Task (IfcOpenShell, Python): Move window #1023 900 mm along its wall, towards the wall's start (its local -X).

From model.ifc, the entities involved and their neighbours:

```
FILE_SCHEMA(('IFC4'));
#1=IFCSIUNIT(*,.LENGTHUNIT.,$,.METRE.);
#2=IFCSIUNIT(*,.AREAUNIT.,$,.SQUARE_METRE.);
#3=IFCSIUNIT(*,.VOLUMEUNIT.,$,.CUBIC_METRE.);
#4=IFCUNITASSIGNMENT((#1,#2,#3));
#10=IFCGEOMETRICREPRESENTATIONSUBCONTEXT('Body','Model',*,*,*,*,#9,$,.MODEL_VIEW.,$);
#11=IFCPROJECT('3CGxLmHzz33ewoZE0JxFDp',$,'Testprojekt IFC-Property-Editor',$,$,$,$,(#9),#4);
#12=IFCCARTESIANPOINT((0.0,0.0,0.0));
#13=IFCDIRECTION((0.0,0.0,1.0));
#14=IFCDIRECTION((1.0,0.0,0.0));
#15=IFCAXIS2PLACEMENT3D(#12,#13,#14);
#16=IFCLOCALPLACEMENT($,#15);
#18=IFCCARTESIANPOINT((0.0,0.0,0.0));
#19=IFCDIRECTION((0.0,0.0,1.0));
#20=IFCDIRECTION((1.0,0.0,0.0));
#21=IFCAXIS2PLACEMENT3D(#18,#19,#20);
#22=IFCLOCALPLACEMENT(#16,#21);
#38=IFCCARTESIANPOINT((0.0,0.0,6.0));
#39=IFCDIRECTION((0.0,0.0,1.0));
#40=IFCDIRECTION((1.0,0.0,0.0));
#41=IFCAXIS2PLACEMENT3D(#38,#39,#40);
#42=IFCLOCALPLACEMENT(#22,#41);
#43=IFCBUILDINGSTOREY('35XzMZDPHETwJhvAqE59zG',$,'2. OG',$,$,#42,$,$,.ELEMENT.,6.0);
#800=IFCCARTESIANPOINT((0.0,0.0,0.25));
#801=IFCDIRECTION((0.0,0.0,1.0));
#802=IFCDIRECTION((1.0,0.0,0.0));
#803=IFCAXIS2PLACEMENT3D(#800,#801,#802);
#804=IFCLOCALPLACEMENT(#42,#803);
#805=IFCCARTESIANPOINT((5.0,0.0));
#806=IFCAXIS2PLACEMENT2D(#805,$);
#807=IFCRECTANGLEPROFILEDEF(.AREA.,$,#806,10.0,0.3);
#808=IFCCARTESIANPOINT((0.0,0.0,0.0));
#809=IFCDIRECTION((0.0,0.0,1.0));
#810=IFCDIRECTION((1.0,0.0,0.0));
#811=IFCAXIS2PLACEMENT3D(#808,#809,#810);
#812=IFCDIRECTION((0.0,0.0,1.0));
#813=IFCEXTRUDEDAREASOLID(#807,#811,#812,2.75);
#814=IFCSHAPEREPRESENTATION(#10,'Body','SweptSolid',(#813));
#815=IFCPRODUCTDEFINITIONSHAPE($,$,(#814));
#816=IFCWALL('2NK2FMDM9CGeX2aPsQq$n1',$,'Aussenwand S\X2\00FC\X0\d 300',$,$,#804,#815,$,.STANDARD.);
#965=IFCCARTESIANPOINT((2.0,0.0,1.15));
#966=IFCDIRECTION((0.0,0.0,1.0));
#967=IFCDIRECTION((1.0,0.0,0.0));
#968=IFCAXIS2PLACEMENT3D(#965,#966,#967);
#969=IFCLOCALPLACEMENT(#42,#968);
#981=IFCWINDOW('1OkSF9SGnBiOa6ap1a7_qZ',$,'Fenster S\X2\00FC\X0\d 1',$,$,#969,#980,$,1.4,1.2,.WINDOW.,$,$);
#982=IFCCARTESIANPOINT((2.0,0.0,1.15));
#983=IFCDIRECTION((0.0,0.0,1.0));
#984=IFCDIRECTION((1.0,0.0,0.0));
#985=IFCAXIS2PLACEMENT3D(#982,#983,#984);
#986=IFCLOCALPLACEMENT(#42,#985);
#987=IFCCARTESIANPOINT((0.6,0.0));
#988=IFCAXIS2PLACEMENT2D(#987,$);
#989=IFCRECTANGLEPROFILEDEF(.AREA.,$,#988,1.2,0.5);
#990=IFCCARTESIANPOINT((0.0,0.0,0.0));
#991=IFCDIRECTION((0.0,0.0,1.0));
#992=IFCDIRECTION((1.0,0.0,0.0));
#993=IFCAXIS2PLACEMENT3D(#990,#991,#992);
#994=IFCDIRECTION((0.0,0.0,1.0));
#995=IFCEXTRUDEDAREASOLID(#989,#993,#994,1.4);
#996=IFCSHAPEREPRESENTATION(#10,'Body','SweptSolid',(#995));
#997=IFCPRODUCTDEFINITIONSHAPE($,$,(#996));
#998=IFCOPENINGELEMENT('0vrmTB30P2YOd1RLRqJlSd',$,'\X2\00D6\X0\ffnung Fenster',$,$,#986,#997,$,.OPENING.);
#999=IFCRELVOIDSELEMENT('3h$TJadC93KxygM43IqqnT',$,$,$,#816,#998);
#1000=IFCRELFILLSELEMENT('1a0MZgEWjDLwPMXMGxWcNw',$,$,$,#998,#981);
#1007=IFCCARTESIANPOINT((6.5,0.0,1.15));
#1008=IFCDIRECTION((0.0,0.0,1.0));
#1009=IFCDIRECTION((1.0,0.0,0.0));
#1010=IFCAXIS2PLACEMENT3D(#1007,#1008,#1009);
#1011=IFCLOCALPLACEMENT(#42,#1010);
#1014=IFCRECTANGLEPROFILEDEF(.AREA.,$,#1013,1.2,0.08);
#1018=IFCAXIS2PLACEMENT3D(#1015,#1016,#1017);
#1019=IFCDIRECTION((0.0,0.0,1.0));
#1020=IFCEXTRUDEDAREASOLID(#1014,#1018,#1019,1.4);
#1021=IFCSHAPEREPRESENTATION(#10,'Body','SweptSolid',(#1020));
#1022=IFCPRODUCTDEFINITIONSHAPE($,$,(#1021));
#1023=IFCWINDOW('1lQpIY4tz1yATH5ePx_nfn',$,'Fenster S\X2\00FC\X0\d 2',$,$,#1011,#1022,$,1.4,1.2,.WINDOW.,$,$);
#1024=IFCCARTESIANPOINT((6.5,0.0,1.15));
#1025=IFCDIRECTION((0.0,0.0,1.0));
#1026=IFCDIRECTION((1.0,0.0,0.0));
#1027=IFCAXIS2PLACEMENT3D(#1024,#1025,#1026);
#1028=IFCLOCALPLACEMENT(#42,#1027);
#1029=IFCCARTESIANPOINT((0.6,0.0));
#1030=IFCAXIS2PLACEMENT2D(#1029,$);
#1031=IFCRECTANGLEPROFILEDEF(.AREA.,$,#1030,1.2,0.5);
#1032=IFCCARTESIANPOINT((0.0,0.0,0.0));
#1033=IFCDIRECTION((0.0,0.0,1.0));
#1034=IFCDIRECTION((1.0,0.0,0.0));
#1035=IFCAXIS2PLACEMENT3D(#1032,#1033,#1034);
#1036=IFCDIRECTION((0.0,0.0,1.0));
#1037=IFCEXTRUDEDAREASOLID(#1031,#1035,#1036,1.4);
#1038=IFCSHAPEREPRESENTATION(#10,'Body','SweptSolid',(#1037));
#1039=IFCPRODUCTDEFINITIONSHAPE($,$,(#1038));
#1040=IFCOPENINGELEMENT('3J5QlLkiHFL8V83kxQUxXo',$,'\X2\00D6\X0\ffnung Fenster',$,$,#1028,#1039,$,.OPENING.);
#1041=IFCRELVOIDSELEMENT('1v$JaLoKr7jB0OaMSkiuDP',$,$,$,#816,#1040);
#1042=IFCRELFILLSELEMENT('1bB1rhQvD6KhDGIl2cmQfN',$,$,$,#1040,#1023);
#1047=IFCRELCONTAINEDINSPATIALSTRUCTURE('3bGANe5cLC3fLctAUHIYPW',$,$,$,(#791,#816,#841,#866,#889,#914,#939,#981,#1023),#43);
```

```python
import ifcopenshell
import ifcopenshell.api.geometry
import ifcopenshell.util.placement

model = ifcopenshell.open("model.ifc")

window = model.by_guid("1lQpIY4tz1yATH5ePx_nfn")
opening = window.FillsVoids[0].RelatingOpeningElement
wall = opening.VoidsElements[0].RelatingBuildingElement

wall_matrix = ifcopenshell.util.placement.get_local_placement(wall.ObjectPlacement)
shift = wall_matrix[:3, 0] * -0.9
before = ifcopenshell.util.placement.get_local_placement(window.ObjectPlacement)[:3, 3].copy()

# The window is not placed relative to its opening, so move both.
for product in (opening, window):
    matrix = ifcopenshell.util.placement.get_local_placement(product.ObjectPlacement)
    matrix[:3, 3] += shift
    ifcopenshell.api.geometry.edit_object_placement(model, product=product, matrix=matrix, is_si=False)

after = ifcopenshell.util.placement.get_local_placement(window.ObjectPlacement)[:3, 3]
print("window moved by", (after - before).round(3) + 0.0)

model.write("model-out.ifc")
```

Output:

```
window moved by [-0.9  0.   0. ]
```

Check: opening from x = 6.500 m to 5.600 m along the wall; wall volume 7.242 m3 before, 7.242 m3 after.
